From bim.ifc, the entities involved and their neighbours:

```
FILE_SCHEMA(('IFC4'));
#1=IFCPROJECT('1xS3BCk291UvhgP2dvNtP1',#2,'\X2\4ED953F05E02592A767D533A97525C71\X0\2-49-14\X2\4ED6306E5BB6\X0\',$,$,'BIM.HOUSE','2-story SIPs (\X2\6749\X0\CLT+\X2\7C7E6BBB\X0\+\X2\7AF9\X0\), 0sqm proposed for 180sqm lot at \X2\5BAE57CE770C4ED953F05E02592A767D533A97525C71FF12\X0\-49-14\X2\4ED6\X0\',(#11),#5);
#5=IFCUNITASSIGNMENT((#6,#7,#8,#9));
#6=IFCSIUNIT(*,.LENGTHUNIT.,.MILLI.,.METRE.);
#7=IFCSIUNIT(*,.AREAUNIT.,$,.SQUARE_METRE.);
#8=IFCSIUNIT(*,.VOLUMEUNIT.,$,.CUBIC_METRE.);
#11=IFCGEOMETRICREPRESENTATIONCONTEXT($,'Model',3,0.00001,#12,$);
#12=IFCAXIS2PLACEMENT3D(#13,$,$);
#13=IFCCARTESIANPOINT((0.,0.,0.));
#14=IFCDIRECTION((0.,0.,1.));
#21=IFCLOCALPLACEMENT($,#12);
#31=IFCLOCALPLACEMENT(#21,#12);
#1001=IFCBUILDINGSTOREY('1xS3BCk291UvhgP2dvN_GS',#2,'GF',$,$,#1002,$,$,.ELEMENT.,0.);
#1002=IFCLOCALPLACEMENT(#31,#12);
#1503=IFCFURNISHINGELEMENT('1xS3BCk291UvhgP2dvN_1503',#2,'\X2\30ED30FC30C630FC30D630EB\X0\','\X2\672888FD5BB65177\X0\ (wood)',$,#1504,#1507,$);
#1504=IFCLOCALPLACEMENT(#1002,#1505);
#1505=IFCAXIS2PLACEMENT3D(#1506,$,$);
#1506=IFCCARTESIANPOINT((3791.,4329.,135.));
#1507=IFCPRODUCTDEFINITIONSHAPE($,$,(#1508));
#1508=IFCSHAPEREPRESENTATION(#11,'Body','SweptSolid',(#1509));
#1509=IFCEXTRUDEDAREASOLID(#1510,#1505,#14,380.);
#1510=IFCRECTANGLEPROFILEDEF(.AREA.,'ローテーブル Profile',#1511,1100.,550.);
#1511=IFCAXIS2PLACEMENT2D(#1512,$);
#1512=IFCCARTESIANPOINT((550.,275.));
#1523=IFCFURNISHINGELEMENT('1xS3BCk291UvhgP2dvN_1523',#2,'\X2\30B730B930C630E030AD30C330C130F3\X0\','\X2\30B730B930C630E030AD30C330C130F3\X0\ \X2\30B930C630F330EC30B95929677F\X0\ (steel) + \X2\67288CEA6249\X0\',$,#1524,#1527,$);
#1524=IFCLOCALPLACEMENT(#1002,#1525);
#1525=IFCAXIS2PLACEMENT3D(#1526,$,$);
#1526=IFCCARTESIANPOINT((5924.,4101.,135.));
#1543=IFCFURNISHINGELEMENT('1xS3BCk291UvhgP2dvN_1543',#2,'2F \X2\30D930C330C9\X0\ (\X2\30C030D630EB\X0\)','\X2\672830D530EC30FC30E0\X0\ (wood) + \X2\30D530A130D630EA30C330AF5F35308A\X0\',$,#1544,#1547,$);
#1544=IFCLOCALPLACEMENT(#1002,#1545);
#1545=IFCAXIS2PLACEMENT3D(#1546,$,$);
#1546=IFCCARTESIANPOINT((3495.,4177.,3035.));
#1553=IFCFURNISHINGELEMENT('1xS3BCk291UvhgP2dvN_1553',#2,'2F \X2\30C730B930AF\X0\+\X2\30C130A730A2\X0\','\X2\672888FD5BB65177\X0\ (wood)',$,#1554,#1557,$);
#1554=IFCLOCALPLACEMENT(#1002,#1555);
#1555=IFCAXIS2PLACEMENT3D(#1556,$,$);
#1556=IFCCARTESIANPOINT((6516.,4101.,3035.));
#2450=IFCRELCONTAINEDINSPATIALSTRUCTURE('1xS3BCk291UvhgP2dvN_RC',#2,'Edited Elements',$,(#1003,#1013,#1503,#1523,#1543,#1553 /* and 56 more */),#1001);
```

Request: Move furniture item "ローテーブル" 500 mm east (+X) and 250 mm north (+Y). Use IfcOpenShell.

```python
import ifcopenshell
import ifcopenshell.api.geometry
import ifcopenshell.util.placement

model = ifcopenshell.open("bim.ifc")

item = model.by_guid("1xS3BCk291UvhgP2dvN_1503")
matrix = ifcopenshell.util.placement.get_local_placement(item.ObjectPlacement)
matrix[0, 3] += 500.0
matrix[1, 3] += 250.0
ifcopenshell.api.geometry.edit_object_placement(model, product=item, matrix=matrix, is_si=False)

print(ifcopenshell.util.placement.get_local_placement(item.ObjectPlacement).round(3) + 0.0)

model.write("bim_edited.ifc")
```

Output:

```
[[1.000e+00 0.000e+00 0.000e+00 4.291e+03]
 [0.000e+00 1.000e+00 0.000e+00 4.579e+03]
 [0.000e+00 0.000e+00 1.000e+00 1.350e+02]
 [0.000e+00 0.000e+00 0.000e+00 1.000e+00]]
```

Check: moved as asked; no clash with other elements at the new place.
